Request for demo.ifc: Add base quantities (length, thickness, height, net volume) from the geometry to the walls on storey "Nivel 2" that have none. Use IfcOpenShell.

First a look at what the model holds.

```python
import ifcopenshell
import ifcopenshell.util.element
import ifcopenshell.util.unit

model = ifcopenshell.open("demo.ifc")
print(model.schema)
for unit_type in ("LENGTHUNIT", "AREAUNIT", "VOLUMEUNIT"):
    print(unit_type, ifcopenshell.util.unit.calculate_unit_scale(model, unit_type))
storey = next(s for s in model.by_type("IfcBuildingStorey") if s.Name == "Nivel 2")
walls = [e for e in ifcopenshell.util.element.get_decomposition(storey) if e.is_a("IfcWall")]
for e in sorted(walls, key=lambda e: e.id()):
    print(e.id(), e.is_a(), e.Name, list(ifcopenshell.util.element.get_psets(e, qtos_only=True)), sep=" | ")
```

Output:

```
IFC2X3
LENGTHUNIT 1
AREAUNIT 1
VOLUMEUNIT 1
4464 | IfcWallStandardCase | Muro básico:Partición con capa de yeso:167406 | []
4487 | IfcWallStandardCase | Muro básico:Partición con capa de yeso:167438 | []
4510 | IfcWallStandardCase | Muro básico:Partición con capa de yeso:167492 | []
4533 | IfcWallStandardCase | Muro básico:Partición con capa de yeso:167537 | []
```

```python
import ifcopenshell
import ifcopenshell.api.pset
import ifcopenshell.geom
import ifcopenshell.util.element
import ifcopenshell.util.shape
import ifcopenshell.util.unit

model = ifcopenshell.open("demo.ifc")
unit_scale = ifcopenshell.util.unit.calculate_unit_scale(model)
volume_scale = ifcopenshell.util.unit.calculate_unit_scale(model, "VOLUMEUNIT")
settings = ifcopenshell.geom.settings()

storey = next(s for s in model.by_type("IfcBuildingStorey") if s.Name == "Nivel 2")
walls = [e for e in ifcopenshell.util.element.get_decomposition(storey) if e.is_a("IfcWall")]

for e in sorted(walls, key=lambda e: e.id()):
    if ifcopenshell.util.element.get_psets(e, qtos_only=True, should_inherit=False):
        continue
    # Geometry comes back in metres, in the element's own axes.
    shape = ifcopenshell.geom.create_shape(settings, e)
    values = {
        "Length": ifcopenshell.util.shape.get_x(shape.geometry) / unit_scale,
        "Width": ifcopenshell.util.shape.get_y(shape.geometry) / unit_scale,
        "Height": ifcopenshell.util.shape.get_z(shape.geometry) / unit_scale,
        "NetVolume": ifcopenshell.util.shape.get_volume(shape.geometry) / volume_scale,
    }
    qto = ifcopenshell.api.pset.add_qto(model, product=e, name="BaseQuantities")
    ifcopenshell.api.pset.edit_qto(model, qto=qto, properties=values)
    print(e.id(), {k: round(v, 3) for k, v in values.items()})

model.write("demo_updated.ifc")
```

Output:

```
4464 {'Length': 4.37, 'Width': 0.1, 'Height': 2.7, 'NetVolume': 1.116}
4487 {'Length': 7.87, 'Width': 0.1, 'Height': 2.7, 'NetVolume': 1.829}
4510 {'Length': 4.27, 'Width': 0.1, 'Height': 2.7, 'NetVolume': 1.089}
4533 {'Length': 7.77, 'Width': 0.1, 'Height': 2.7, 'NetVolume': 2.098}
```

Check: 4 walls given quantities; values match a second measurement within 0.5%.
